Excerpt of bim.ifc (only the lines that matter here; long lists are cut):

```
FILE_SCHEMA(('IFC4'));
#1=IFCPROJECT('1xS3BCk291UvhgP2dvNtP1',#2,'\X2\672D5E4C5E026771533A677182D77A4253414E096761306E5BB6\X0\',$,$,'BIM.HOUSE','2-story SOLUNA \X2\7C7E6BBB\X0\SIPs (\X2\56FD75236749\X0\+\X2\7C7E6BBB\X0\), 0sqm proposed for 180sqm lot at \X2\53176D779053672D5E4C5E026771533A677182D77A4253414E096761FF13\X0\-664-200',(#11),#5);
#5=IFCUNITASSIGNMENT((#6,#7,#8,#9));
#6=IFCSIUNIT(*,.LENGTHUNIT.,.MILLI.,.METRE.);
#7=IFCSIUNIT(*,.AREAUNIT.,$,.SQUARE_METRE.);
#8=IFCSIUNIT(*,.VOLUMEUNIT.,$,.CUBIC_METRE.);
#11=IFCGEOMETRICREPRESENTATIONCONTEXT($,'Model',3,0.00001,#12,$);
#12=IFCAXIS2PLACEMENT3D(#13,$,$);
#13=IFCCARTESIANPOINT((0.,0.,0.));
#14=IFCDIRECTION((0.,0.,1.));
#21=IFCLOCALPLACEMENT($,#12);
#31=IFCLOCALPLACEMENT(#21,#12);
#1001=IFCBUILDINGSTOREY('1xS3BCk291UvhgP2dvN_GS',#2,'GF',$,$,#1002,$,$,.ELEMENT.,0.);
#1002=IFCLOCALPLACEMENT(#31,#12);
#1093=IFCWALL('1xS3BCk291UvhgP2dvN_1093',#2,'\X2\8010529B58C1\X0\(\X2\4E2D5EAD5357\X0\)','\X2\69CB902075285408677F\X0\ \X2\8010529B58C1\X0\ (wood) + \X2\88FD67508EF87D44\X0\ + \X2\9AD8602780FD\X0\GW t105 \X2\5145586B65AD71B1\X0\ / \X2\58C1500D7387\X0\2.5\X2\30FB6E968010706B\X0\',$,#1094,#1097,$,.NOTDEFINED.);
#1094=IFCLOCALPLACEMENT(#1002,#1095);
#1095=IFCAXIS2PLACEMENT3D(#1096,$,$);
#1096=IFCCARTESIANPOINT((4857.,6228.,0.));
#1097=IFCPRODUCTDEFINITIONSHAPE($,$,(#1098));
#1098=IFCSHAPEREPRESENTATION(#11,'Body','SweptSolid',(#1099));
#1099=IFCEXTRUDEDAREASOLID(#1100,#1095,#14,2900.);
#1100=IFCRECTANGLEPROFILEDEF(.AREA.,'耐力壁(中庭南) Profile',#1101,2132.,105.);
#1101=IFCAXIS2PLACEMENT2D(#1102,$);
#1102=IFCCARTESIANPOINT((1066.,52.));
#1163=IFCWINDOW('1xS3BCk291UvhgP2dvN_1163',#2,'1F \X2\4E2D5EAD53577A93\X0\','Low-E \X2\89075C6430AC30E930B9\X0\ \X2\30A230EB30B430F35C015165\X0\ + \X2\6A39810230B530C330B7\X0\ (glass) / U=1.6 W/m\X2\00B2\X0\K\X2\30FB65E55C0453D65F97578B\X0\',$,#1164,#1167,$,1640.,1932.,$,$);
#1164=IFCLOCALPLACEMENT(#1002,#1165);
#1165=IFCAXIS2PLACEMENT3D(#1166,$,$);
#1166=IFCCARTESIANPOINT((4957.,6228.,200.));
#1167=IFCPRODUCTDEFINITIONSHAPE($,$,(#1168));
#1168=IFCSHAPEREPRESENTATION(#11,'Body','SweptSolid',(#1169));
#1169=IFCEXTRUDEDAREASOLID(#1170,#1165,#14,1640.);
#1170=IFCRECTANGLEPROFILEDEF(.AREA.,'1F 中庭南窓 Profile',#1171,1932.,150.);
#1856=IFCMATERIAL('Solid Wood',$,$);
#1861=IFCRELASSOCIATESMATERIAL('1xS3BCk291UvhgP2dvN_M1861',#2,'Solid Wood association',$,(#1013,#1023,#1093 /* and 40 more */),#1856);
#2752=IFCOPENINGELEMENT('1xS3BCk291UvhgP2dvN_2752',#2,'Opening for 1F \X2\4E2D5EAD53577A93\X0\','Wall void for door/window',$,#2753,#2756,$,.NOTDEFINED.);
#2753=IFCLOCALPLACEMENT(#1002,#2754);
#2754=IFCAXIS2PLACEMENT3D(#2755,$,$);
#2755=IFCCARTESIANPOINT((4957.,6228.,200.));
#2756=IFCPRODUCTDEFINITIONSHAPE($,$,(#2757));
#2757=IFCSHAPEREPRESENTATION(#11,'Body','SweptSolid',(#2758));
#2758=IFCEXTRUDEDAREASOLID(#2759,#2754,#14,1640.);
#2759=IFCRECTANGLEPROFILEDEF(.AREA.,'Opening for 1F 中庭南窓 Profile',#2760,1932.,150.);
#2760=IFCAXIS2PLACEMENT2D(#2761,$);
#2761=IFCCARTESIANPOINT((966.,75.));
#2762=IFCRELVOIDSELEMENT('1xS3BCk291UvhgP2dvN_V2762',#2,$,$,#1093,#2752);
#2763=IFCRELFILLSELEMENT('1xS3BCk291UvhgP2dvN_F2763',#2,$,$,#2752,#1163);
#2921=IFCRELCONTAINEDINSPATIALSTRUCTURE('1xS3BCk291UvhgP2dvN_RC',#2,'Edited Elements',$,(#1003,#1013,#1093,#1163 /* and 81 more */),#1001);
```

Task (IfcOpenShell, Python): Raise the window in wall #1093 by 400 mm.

```python
import numpy as np
import ifcopenshell
import ifcopenshell.api.geometry
import ifcopenshell.util.placement
import ifcopenshell.util.unit

model = ifcopenshell.open("bim.ifc")
unit_scale = ifcopenshell.util.unit.calculate_unit_scale(model)

window = model.by_guid("1xS3BCk291UvhgP2dvN_1163")
opening = window.FillsVoids[0].RelatingOpeningElement
dz = 400.0

shift = np.array([0.0, 0.0, dz])
# The window is not placed relative to its opening, so move both.
for product in (opening, window):
    matrix = ifcopenshell.util.placement.get_local_placement(product.ObjectPlacement)
    matrix[:3, 3] += shift
    ifcopenshell.api.geometry.edit_object_placement(model, product=product, matrix=matrix, is_si=False)

print(f"moved by {dz * unit_scale:+.3f} m")

model.write("bim_rev.ifc")
```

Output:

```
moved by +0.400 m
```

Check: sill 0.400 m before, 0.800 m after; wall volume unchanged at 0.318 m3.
